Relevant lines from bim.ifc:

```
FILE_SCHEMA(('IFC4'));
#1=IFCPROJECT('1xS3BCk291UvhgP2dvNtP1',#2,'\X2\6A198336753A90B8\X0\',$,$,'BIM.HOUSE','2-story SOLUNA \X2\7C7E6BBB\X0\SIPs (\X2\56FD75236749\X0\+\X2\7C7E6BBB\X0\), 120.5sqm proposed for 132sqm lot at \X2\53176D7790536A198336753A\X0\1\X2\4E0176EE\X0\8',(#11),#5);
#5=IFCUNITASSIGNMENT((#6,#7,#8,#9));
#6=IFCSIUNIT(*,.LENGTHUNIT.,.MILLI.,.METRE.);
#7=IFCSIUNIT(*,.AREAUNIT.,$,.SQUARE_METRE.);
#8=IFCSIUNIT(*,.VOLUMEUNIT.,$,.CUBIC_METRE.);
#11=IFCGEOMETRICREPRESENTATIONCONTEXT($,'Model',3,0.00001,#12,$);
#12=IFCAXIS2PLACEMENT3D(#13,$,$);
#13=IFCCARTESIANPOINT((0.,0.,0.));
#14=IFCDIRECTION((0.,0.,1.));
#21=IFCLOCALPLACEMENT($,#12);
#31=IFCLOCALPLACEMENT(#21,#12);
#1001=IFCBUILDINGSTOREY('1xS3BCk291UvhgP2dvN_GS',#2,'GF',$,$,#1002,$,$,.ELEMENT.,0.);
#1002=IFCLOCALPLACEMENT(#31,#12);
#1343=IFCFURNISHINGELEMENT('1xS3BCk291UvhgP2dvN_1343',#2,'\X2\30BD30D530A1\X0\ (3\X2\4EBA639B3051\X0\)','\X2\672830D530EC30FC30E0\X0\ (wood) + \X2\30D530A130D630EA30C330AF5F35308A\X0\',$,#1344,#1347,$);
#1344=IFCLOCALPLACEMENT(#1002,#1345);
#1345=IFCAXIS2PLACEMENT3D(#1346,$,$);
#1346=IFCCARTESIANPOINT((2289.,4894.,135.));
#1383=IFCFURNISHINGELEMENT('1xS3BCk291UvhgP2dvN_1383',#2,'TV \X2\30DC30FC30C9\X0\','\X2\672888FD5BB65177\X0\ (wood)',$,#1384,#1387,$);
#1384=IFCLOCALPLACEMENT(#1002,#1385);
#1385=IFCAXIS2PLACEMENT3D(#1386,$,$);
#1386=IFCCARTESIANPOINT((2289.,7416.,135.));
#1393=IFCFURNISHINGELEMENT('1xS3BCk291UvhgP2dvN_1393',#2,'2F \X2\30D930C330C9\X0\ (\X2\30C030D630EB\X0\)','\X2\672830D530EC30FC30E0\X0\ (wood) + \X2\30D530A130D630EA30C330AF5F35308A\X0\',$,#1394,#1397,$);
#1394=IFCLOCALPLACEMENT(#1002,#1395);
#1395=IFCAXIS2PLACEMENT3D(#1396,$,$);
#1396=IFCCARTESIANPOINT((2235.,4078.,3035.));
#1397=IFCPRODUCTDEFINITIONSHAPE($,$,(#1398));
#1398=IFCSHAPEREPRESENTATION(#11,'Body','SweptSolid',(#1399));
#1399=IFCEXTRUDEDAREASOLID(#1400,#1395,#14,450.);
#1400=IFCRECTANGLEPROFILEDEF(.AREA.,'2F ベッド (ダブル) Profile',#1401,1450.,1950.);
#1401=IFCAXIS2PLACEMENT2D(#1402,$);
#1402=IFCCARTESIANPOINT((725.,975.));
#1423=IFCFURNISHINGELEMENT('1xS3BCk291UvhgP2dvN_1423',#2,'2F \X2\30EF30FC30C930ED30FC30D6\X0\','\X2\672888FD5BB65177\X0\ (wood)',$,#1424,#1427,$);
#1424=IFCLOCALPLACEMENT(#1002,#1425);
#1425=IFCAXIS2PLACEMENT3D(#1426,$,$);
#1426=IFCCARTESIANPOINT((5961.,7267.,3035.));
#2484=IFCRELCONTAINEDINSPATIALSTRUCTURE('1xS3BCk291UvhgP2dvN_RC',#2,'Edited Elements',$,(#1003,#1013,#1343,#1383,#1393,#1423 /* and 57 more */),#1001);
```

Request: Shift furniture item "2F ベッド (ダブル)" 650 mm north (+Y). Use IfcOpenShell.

```python
import ifcopenshell
import ifcopenshell.api.geometry
import ifcopenshell.util.placement
import ifcopenshell.util.unit

model = ifcopenshell.open("bim.ifc")
unit_scale = ifcopenshell.util.unit.calculate_unit_scale(model)

item = model.by_id(1393)
matrix = ifcopenshell.util.placement.get_local_placement(item.ObjectPlacement)
matrix[1, 3] += 0.65 / unit_scale
ifcopenshell.api.geometry.edit_object_placement(model, product=item, matrix=matrix, is_si=False)

print(ifcopenshell.util.placement.get_local_placement(item.ObjectPlacement).round(3) + 0.0)

model.write("bim_rev.ifc")
```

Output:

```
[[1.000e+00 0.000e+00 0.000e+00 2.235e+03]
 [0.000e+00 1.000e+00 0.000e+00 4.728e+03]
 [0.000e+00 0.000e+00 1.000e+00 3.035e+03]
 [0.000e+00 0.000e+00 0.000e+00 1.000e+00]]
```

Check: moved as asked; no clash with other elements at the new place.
